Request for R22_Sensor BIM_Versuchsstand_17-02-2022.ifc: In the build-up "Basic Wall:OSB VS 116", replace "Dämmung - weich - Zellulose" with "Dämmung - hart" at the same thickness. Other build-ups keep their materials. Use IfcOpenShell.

First a look at what the model holds.

```python
import ifcopenshell
import ifcopenshell.util.element

model = ifcopenshell.open("R22_Sensor BIM_Versuchsstand_17-02-2022.ifc")
print(model.schema)
for layer_set in model.by_type("IfcMaterialLayerSet"):
    if layer_set.LayerSetName == "Basic Wall:OSB VS 116":
        for layer in layer_set.MaterialLayers:
            print(layer.id(), layer.Material and layer.Material.Name, layer.LayerThickness, sep=" | ")
        print(len(ifcopenshell.util.element.get_elements_by_material(model, layer_set)), "elements and types use it")
print(sorted(m.Name for m in model.by_type("IfcMaterial") if m.Name)[:60])
```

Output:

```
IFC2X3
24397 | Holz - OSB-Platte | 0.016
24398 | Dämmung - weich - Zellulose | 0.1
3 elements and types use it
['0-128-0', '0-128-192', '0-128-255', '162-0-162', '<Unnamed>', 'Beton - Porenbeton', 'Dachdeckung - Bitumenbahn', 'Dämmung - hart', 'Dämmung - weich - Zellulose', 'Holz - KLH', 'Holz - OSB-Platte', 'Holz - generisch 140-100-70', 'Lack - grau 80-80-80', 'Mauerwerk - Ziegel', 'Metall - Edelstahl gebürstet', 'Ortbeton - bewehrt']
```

```python
import ifcopenshell
import ifcopenshell.api.material

model = ifcopenshell.open("R22_Sensor BIM_Versuchsstand_17-02-2022.ifc")

layer_set = next(s for s in model.by_type("IfcMaterialLayerSet") if s.LayerSetName == "Basic Wall:OSB VS 116")
layer = next(l for l in layer_set.MaterialLayers if l.Material and l.Material.Name == "Dämmung - weich - Zellulose")
material = next(m for m in model.by_type("IfcMaterial") if m.Name == "Dämmung - hart")

# Point this one layer at the other material; renaming the old one would change it everywhere.
ifcopenshell.api.material.edit_layer(model, layer=layer, attributes={}, material=material)

print([l.Material.Name if l.Material else None for l in layer_set.MaterialLayers])

model.write("R22_Sensor BIM_Versuchsstand_17-02-2022_rev.ifc")
```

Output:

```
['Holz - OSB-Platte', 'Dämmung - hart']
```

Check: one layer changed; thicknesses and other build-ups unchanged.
